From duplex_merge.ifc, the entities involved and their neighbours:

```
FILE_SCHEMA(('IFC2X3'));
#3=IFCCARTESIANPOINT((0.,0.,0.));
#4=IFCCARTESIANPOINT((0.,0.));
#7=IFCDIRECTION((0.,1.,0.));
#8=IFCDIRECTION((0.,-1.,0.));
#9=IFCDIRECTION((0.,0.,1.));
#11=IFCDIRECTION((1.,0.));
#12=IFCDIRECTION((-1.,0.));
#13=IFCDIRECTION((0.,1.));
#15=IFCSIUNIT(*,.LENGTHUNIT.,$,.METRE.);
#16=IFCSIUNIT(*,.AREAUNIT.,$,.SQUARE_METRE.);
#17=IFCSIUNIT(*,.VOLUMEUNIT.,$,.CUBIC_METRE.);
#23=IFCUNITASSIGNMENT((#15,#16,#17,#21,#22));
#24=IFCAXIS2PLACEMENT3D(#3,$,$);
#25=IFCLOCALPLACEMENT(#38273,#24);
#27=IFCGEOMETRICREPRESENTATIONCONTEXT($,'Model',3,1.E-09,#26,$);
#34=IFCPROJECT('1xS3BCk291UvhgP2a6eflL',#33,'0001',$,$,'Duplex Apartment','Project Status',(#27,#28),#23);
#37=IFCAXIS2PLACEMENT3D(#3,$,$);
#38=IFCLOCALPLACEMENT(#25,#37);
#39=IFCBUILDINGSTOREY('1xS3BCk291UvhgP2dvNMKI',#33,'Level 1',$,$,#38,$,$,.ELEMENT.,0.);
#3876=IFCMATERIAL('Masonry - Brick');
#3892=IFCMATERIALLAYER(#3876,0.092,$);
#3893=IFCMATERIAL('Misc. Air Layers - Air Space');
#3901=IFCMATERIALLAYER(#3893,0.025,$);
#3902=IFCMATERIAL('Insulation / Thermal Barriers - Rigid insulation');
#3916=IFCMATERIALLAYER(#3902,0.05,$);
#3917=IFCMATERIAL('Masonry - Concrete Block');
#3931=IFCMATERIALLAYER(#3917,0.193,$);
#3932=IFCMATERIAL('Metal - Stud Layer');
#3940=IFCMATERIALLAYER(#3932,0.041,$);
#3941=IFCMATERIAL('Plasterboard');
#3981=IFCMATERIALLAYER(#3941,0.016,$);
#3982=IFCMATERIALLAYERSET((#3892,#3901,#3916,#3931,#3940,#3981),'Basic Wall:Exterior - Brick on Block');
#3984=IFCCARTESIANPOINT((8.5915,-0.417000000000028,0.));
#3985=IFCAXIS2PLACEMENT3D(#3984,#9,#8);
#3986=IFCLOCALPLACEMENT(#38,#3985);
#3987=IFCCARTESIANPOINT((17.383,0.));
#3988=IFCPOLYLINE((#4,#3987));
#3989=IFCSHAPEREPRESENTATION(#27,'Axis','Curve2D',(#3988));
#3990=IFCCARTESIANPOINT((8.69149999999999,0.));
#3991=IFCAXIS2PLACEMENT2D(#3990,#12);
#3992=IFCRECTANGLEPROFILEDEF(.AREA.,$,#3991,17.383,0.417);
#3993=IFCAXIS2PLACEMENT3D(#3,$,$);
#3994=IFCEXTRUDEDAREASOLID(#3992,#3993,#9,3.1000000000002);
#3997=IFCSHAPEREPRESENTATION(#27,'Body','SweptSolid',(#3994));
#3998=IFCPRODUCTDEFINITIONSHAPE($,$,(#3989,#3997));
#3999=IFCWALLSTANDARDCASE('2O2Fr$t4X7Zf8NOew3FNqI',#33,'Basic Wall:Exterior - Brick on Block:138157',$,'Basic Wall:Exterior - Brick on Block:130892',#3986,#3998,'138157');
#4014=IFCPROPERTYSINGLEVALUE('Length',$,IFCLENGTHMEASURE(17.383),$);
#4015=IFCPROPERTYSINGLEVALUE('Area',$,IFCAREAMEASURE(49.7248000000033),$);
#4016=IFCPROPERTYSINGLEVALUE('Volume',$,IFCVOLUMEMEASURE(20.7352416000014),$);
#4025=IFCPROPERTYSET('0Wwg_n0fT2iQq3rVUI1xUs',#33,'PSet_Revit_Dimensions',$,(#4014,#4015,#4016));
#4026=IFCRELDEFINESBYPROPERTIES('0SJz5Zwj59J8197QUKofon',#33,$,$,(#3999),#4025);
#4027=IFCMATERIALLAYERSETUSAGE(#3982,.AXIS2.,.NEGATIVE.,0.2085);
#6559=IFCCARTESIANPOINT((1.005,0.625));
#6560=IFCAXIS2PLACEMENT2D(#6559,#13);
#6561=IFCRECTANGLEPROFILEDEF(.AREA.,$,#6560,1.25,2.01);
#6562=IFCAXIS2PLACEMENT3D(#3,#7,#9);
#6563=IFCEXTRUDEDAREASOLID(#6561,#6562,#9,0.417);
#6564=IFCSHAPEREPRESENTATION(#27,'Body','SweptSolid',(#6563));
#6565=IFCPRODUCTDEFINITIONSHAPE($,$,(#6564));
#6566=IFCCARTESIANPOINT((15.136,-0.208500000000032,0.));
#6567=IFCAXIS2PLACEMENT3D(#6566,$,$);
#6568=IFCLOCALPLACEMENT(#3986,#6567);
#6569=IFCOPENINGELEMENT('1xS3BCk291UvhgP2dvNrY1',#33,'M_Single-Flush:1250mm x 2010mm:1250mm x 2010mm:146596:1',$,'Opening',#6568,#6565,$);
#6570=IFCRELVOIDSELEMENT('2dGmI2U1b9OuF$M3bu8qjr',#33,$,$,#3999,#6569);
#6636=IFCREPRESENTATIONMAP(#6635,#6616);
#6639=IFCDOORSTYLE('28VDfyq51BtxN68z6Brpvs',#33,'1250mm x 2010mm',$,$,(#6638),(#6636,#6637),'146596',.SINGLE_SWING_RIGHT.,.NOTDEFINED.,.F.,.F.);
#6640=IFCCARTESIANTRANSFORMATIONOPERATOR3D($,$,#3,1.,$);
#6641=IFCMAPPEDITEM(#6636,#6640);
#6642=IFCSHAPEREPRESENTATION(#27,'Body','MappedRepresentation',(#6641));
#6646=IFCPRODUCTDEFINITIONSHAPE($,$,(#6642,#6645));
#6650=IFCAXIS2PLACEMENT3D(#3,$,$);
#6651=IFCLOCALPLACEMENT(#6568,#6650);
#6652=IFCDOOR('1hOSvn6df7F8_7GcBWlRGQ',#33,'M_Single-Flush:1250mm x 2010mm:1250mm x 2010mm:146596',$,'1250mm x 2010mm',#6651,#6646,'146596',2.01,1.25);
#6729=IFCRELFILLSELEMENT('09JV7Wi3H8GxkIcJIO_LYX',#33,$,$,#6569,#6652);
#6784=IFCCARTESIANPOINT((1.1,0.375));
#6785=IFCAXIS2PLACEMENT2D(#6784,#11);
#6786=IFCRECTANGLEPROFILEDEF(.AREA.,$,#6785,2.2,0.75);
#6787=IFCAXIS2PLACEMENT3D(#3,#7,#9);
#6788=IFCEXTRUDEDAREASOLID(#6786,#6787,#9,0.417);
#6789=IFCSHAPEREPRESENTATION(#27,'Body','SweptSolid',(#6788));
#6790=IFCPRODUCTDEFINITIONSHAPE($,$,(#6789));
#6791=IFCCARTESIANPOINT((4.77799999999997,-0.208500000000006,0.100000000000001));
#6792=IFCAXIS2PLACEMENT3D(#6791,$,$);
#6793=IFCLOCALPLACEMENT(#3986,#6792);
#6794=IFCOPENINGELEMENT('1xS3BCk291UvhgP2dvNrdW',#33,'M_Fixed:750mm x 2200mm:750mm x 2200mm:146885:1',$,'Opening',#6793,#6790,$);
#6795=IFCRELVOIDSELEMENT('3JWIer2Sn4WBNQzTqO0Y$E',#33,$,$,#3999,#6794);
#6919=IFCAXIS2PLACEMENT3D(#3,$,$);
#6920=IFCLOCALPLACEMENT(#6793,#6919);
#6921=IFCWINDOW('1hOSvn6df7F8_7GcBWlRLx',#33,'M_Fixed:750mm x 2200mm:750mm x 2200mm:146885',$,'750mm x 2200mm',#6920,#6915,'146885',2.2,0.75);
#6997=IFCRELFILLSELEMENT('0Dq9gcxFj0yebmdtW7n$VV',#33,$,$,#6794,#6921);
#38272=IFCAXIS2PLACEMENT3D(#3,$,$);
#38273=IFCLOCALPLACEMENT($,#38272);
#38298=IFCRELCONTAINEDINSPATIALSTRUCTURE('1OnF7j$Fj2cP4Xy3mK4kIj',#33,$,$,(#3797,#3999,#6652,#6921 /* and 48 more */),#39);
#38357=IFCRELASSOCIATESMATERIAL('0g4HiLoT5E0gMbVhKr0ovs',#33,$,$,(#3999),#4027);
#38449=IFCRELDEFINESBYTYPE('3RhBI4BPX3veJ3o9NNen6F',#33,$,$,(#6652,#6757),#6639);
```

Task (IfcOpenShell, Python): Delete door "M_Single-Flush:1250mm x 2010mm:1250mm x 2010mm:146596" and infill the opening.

```python
import ifcopenshell
import ifcopenshell.api.feature
import ifcopenshell.api.pset
import ifcopenshell.api.root
import ifcopenshell.geom
import ifcopenshell.util.element
import ifcopenshell.util.shape
import ifcopenshell.util.unit

model = ifcopenshell.open("duplex_merge.ifc")
area_scale = ifcopenshell.util.unit.calculate_unit_scale(model, "AREAUNIT")
volume_scale = ifcopenshell.util.unit.calculate_unit_scale(model, "VOLUMEUNIT")
settings = ifcopenshell.geom.settings()


def volume(element):
    """Net volume in cubic metres, openings subtracted."""
    shape = ifcopenshell.geom.create_shape(settings, element)
    return ifcopenshell.util.shape.get_volume(shape.geometry)


door = model.by_id(6652)
opening = door.FillsVoids[0].RelatingOpeningElement
wall = opening.VoidsElements[0].RelatingBuildingElement
before = volume(wall)

ifcopenshell.api.root.remove_product(model, product=door)
ifcopenshell.api.feature.remove_feature(model, feature=opening)

after = volume(wall)
thickness = 0.417  # wall thickness in metres

# Update the wall's stored quantities.
pset = model.by_id(ifcopenshell.util.element.get_pset(wall, "PSet_Revit_Dimensions", should_inherit=False)["id"])
ifcopenshell.api.pset.edit_pset(model, pset=pset, properties={
    "Area": model.create_entity("IfcAreaMeasure", after / thickness / area_scale),
    "Volume": model.create_entity("IfcVolumeMeasure", after / volume_scale),
})

print(f"wall volume {before:.3f} -> {after:.3f} m3")

model.write("duplex_merge_v2.ifc")
```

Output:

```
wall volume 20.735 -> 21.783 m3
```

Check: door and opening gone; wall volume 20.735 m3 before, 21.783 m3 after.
